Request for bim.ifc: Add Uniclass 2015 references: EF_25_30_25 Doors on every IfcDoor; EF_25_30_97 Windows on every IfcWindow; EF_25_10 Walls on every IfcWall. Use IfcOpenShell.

First a look at what the model holds.

```python
import ifcopenshell

model = ifcopenshell.open("bim.ifc")
print(model.schema)
print("classifications:", [c.Name for c in model.by_type("IfcClassification")])
for ifc_class in ("IfcDoor", "IfcRoof", "IfcStair", "IfcWall", "IfcWindow"):
    print(ifc_class, len(model.by_type(ifc_class)))
```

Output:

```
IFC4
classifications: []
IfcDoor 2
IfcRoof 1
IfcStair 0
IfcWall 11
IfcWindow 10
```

```python
import ifcopenshell
import ifcopenshell.api.classification

model = ifcopenshell.open("bim.ifc")

system = ifcopenshell.api.classification.add_classification(model, classification="Uniclass 2015")

codes = {
    "IfcDoor": ("EF_25_30_25", "Doors"),
    "IfcWindow": ("EF_25_30_97", "Windows"),
    "IfcWall": ("EF_25_10", "Walls"),
}
for ifc_class, (code, name) in codes.items():
    products = model.by_type(ifc_class)
    ifcopenshell.api.classification.add_reference(
        model, products=products, classification=system, identification=code, name=name
    )
    print(code, len(products))

model.write("bim_rev.ifc")
```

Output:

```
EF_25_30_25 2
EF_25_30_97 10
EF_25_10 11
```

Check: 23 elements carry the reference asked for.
